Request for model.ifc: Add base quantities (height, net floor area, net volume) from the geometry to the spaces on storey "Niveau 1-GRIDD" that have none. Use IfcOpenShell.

First a look at what the model holds.

```python
import ifcopenshell
import ifcopenshell.util.element
import ifcopenshell.util.unit

model = ifcopenshell.open("model.ifc")
print(model.schema)
for unit_type in ("LENGTHUNIT", "AREAUNIT", "VOLUMEUNIT"):
    print(unit_type, ifcopenshell.util.unit.calculate_unit_scale(model, unit_type))
storey = next(s for s in model.by_type("IfcBuildingStorey") if s.Name == "Niveau 1-GRIDD")
spaces = [e for e in ifcopenshell.util.element.get_decomposition(storey) if e.is_a("IfcSpace")]
for e in sorted(spaces, key=lambda e: e.id()):
    print(e.id(), e.is_a(), e.Name, list(ifcopenshell.util.element.get_psets(e, qtos_only=True)), sep=" | ")
```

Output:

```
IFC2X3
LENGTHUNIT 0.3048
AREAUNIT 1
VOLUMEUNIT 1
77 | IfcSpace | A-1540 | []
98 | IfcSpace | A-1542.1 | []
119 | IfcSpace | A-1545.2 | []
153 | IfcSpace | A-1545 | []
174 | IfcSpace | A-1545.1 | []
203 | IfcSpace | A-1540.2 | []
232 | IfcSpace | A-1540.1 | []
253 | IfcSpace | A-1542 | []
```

```python
import ifcopenshell
import ifcopenshell.api.pset
import ifcopenshell.geom
import ifcopenshell.util.element
import ifcopenshell.util.shape
import ifcopenshell.util.unit

model = ifcopenshell.open("model.ifc")
unit_scale = ifcopenshell.util.unit.calculate_unit_scale(model)
area_scale = ifcopenshell.util.unit.calculate_unit_scale(model, "AREAUNIT")
volume_scale = ifcopenshell.util.unit.calculate_unit_scale(model, "VOLUMEUNIT")
settings = ifcopenshell.geom.settings()

storey = next(s for s in model.by_type("IfcBuildingStorey") if s.Name == "Niveau 1-GRIDD")
spaces = [e for e in ifcopenshell.util.element.get_decomposition(storey) if e.is_a("IfcSpace")]

for e in sorted(spaces, key=lambda e: e.id()):
    if ifcopenshell.util.element.get_psets(e, qtos_only=True, should_inherit=False):
        continue
    # Geometry comes back in metres, in the element's own axes.
    shape = ifcopenshell.geom.create_shape(settings, e)
    values = {
        "Height": ifcopenshell.util.shape.get_z(shape.geometry) / unit_scale,
        "NetFloorArea": ifcopenshell.util.shape.get_footprint_area(shape.geometry) / area_scale,
        "NetVolume": ifcopenshell.util.shape.get_volume(shape.geometry) / volume_scale,
    }
    qto = ifcopenshell.api.pset.add_qto(model, product=e, name="BaseQuantities")
    ifcopenshell.api.pset.edit_qto(model, qto=qto, properties=values)
    print(e.id(), {k: round(v, 3) for k, v in values.items()})

model.write("model-out.ifc")
```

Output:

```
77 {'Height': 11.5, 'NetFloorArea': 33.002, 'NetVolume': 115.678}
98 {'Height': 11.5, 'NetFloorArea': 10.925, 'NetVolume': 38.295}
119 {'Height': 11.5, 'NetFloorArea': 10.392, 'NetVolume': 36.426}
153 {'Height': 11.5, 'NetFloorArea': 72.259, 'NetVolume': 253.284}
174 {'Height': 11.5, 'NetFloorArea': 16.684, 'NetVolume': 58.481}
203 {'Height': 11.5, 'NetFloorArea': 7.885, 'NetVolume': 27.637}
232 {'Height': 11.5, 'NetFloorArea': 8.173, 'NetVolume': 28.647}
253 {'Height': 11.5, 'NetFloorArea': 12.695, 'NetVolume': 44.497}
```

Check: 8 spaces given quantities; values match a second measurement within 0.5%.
